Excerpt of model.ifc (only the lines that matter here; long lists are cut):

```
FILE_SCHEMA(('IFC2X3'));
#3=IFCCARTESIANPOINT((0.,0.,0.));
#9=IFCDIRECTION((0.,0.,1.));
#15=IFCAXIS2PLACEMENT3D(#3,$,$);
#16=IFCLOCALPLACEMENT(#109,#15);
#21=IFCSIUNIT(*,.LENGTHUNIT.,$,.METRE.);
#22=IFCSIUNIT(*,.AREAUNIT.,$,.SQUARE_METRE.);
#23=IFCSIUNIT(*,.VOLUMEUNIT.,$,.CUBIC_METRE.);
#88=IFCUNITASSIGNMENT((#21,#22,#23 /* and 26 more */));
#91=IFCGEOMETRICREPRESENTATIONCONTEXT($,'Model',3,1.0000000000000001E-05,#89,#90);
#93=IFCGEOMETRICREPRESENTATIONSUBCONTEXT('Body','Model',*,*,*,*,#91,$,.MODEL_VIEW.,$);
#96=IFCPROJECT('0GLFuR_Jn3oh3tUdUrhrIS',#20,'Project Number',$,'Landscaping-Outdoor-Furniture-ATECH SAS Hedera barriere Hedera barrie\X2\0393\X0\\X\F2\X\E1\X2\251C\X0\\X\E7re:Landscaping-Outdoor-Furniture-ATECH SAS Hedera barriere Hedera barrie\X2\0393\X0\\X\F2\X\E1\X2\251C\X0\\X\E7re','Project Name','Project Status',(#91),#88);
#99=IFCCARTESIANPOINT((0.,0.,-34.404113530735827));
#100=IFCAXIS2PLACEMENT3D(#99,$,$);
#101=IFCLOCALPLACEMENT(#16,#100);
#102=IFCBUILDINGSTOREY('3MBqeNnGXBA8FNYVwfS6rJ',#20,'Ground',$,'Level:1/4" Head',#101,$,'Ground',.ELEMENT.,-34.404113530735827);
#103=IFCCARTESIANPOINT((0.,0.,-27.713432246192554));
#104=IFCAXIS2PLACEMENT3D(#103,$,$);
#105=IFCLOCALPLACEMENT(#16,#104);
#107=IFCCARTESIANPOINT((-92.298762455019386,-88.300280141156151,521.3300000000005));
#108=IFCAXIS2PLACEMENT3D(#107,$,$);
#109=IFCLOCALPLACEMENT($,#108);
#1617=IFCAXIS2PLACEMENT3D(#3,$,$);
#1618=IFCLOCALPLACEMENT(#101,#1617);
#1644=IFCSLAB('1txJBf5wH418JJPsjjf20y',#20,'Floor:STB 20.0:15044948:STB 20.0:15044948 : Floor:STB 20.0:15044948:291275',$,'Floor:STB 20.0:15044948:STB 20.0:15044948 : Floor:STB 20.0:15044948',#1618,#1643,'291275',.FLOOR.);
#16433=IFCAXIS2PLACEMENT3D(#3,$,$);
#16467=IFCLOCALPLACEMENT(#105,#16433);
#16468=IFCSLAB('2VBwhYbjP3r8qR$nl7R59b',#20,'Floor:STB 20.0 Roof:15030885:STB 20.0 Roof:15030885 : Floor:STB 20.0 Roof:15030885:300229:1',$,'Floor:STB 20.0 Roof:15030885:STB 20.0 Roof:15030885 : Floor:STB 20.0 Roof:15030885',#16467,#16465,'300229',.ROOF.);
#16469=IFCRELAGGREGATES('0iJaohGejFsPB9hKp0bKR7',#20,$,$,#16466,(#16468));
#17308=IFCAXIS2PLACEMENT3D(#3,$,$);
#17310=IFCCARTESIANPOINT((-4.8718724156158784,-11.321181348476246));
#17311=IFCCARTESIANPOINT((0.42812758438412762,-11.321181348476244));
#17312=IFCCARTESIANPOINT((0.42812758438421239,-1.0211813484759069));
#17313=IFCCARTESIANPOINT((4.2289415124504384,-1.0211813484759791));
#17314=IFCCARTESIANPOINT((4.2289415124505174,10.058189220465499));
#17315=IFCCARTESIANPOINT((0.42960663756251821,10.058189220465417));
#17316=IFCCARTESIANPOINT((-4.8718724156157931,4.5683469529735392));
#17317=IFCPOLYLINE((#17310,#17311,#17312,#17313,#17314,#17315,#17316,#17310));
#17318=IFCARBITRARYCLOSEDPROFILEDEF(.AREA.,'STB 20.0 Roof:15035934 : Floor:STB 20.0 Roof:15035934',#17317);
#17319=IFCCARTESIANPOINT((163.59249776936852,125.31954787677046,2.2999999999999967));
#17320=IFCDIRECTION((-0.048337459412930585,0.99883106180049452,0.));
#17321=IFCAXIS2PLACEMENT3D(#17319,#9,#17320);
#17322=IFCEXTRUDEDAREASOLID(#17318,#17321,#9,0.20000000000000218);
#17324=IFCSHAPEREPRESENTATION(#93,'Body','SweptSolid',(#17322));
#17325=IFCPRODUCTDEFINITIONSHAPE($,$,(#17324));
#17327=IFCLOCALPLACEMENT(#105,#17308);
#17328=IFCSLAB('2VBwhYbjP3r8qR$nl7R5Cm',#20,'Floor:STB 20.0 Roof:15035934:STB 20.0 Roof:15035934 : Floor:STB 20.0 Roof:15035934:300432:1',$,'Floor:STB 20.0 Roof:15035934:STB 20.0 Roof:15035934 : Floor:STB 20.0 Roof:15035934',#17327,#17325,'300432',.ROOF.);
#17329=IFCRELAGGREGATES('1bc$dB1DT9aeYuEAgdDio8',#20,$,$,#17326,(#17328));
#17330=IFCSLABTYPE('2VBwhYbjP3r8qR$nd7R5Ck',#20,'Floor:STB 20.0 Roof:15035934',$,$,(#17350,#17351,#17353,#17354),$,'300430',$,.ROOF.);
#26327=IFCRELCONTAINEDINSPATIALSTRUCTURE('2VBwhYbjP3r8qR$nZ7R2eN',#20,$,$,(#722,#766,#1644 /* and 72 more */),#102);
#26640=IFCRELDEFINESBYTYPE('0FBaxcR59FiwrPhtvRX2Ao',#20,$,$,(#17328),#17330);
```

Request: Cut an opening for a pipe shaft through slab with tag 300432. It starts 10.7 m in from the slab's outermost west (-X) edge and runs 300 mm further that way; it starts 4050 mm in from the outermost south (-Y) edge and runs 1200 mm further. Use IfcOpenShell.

```python
import numpy as np
import ifcopenshell
import ifcopenshell.api.feature
import ifcopenshell.api.geometry
import ifcopenshell.api.root
import ifcopenshell.geom
import ifcopenshell.util.placement
import ifcopenshell.util.representation
import ifcopenshell.util.shape
import ifcopenshell.util.unit

model = ifcopenshell.open("model.ifc")
unit_scale = ifcopenshell.util.unit.calculate_unit_scale(model)
settings = ifcopenshell.geom.settings()


def volume(element):
    """Net volume in cubic metres, openings subtracted."""
    shape = ifcopenshell.geom.create_shape(settings, element)
    return ifcopenshell.util.shape.get_volume(shape.geometry)


slab = model.by_id(17328)
before = volume(slab)

# Extent in the slab's own axes, in metres. The edges named are its -X and -Y sides.
slab_shape = ifcopenshell.geom.create_shape(settings, slab)
vertices = ifcopenshell.util.shape.get_vertices(slab_shape.geometry)
x_min, y_min, bottom = vertices.min(axis=0)
top = vertices[:, 2].max()

opening = ifcopenshell.api.root.create_entity(model, ifc_class="IfcOpeningElement", name="Pipe shaft opening")
context = ifcopenshell.util.representation.get_context(model, "Model", "Body", "MODEL_VIEW")
width, depth = 0.3, 1.2
outline = [(0.0, 0.0), (width, 0.0), (width, depth), (0.0, depth), (0.0, 0.0)]
# Overshoot both faces by 50 mm so the cut is clean.
shape = ifcopenshell.api.geometry.add_slab_representation(
    model, context=context, depth=top - bottom + 0.1, polyline=outline
)
ifcopenshell.api.geometry.assign_representation(model, product=opening, representation=shape)

matrix = ifcopenshell.util.placement.get_local_placement(slab.ObjectPlacement)
matrix[:, 3] = matrix @ np.append(np.array([x_min + 10.7, y_min + 4.05, bottom - 0.05]) / unit_scale, 1.0)
ifcopenshell.api.geometry.edit_object_placement(model, product=opening, matrix=matrix, is_si=False)
ifcopenshell.api.feature.add_feature(model, feature=opening, element=slab)

after = volume(slab)

print(f"slab volume {before:.3f} -> {after:.3f} m3")

model.write("model_updated.ifc")
```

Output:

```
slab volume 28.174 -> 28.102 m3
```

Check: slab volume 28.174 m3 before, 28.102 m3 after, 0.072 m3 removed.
